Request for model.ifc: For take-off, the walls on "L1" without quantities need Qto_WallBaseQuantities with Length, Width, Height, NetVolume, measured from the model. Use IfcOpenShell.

First a look at what the model holds.

```python
import ifcopenshell
import ifcopenshell.util.element
import ifcopenshell.util.unit

model = ifcopenshell.open("model.ifc")
print(model.schema)
for unit_type in ("LENGTHUNIT", "AREAUNIT", "VOLUMEUNIT"):
    print(unit_type, ifcopenshell.util.unit.calculate_unit_scale(model, unit_type))
storey = next(s for s in model.by_type("IfcBuildingStorey") if s.Name == "L1")
walls = [e for e in ifcopenshell.util.element.get_decomposition(storey) if e.is_a("IfcWall")]
for e in sorted(walls, key=lambda e: e.id()):
    print(e.id(), e.is_a(), e.Name, list(ifcopenshell.util.element.get_psets(e, qtos_only=True)), sep=" | ")
```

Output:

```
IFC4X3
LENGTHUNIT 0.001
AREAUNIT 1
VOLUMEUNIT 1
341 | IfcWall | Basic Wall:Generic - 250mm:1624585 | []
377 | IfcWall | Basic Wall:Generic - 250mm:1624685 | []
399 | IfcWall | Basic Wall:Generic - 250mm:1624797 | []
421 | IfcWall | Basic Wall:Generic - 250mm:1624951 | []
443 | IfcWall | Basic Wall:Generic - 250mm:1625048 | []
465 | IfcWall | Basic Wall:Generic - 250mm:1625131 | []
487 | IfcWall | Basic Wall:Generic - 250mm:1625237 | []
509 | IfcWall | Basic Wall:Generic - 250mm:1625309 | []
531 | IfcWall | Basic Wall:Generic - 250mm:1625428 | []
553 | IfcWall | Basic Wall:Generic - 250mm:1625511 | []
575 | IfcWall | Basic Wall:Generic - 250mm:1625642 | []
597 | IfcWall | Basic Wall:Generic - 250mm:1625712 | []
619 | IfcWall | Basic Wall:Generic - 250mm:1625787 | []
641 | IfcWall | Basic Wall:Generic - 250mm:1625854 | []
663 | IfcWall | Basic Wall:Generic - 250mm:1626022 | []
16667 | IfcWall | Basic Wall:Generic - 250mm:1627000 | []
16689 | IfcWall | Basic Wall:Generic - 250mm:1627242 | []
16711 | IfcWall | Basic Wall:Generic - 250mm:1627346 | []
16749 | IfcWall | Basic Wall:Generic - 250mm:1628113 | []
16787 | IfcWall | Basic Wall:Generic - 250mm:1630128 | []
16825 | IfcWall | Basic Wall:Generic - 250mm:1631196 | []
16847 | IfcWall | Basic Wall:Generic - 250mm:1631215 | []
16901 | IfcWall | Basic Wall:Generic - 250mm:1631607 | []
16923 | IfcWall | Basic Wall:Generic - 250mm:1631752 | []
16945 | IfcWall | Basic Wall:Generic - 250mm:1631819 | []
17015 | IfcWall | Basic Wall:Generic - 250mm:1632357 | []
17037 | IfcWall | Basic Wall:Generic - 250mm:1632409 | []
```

```python
import ifcopenshell
import ifcopenshell.api.pset
import ifcopenshell.geom
import ifcopenshell.util.element
import ifcopenshell.util.shape
import ifcopenshell.util.unit

model = ifcopenshell.open("model.ifc")
unit_scale = ifcopenshell.util.unit.calculate_unit_scale(model)
volume_scale = ifcopenshell.util.unit.calculate_unit_scale(model, "VOLUMEUNIT")
settings = ifcopenshell.geom.settings()

storey = next(s for s in model.by_type("IfcBuildingStorey") if s.Name == "L1")
walls = [e for e in ifcopenshell.util.element.get_decomposition(storey) if e.is_a("IfcWall")]

for e in sorted(walls, key=lambda e: e.id()):
    if ifcopenshell.util.element.get_psets(e, qtos_only=True, should_inherit=False):
        continue
    # Geometry comes back in metres, in the element's own axes.
    shape = ifcopenshell.geom.create_shape(settings, e)
    values = {
        "Length": ifcopenshell.util.shape.get_x(shape.geometry) / unit_scale,
        "Width": ifcopenshell.util.shape.get_y(shape.geometry) / unit_scale,
        "Height": ifcopenshell.util.shape.get_z(shape.geometry) / unit_scale,
        "NetVolume": ifcopenshell.util.shape.get_volume(shape.geometry) / volume_scale,
    }
    qto = ifcopenshell.api.pset.add_qto(model, product=e, name="Qto_WallBaseQuantities")
    ifcopenshell.api.pset.edit_qto(model, qto=qto, properties=values)
    print(e.id(), {k: round(v, 3) for k, v in values.items()})

model.write("model-out.ifc")
```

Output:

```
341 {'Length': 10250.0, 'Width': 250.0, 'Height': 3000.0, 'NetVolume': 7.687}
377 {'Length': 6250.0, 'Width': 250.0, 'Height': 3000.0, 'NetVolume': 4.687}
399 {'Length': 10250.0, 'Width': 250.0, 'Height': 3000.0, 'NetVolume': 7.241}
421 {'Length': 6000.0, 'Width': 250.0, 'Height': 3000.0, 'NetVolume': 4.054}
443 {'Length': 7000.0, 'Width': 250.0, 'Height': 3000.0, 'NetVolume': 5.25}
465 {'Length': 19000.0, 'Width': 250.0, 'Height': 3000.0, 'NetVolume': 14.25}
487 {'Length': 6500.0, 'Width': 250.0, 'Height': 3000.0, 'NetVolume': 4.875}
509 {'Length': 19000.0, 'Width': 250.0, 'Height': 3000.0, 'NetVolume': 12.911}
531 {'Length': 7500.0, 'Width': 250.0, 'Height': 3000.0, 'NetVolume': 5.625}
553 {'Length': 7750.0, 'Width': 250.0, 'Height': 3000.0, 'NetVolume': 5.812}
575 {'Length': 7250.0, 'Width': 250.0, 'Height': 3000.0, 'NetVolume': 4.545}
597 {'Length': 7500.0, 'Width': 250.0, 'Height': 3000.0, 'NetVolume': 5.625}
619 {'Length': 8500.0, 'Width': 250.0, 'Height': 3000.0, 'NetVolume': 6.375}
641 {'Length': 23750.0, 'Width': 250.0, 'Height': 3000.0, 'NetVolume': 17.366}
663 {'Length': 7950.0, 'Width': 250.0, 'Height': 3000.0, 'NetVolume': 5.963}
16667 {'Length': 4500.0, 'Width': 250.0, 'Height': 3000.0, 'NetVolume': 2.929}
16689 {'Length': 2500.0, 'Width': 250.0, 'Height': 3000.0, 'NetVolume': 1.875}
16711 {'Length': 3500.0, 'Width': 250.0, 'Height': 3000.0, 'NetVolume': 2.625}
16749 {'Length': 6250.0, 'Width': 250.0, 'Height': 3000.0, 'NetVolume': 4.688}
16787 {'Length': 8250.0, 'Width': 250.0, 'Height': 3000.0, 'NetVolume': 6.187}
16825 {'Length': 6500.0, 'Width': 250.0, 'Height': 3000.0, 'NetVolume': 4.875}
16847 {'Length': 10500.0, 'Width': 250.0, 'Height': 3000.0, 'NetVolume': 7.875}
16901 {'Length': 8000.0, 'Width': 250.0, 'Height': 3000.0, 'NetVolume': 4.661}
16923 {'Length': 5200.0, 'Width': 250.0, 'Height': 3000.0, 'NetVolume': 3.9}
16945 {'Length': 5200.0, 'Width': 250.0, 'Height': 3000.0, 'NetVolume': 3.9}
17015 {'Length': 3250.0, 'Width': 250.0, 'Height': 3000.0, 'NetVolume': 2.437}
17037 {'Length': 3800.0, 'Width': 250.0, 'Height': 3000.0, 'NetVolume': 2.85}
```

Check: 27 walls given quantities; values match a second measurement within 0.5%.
